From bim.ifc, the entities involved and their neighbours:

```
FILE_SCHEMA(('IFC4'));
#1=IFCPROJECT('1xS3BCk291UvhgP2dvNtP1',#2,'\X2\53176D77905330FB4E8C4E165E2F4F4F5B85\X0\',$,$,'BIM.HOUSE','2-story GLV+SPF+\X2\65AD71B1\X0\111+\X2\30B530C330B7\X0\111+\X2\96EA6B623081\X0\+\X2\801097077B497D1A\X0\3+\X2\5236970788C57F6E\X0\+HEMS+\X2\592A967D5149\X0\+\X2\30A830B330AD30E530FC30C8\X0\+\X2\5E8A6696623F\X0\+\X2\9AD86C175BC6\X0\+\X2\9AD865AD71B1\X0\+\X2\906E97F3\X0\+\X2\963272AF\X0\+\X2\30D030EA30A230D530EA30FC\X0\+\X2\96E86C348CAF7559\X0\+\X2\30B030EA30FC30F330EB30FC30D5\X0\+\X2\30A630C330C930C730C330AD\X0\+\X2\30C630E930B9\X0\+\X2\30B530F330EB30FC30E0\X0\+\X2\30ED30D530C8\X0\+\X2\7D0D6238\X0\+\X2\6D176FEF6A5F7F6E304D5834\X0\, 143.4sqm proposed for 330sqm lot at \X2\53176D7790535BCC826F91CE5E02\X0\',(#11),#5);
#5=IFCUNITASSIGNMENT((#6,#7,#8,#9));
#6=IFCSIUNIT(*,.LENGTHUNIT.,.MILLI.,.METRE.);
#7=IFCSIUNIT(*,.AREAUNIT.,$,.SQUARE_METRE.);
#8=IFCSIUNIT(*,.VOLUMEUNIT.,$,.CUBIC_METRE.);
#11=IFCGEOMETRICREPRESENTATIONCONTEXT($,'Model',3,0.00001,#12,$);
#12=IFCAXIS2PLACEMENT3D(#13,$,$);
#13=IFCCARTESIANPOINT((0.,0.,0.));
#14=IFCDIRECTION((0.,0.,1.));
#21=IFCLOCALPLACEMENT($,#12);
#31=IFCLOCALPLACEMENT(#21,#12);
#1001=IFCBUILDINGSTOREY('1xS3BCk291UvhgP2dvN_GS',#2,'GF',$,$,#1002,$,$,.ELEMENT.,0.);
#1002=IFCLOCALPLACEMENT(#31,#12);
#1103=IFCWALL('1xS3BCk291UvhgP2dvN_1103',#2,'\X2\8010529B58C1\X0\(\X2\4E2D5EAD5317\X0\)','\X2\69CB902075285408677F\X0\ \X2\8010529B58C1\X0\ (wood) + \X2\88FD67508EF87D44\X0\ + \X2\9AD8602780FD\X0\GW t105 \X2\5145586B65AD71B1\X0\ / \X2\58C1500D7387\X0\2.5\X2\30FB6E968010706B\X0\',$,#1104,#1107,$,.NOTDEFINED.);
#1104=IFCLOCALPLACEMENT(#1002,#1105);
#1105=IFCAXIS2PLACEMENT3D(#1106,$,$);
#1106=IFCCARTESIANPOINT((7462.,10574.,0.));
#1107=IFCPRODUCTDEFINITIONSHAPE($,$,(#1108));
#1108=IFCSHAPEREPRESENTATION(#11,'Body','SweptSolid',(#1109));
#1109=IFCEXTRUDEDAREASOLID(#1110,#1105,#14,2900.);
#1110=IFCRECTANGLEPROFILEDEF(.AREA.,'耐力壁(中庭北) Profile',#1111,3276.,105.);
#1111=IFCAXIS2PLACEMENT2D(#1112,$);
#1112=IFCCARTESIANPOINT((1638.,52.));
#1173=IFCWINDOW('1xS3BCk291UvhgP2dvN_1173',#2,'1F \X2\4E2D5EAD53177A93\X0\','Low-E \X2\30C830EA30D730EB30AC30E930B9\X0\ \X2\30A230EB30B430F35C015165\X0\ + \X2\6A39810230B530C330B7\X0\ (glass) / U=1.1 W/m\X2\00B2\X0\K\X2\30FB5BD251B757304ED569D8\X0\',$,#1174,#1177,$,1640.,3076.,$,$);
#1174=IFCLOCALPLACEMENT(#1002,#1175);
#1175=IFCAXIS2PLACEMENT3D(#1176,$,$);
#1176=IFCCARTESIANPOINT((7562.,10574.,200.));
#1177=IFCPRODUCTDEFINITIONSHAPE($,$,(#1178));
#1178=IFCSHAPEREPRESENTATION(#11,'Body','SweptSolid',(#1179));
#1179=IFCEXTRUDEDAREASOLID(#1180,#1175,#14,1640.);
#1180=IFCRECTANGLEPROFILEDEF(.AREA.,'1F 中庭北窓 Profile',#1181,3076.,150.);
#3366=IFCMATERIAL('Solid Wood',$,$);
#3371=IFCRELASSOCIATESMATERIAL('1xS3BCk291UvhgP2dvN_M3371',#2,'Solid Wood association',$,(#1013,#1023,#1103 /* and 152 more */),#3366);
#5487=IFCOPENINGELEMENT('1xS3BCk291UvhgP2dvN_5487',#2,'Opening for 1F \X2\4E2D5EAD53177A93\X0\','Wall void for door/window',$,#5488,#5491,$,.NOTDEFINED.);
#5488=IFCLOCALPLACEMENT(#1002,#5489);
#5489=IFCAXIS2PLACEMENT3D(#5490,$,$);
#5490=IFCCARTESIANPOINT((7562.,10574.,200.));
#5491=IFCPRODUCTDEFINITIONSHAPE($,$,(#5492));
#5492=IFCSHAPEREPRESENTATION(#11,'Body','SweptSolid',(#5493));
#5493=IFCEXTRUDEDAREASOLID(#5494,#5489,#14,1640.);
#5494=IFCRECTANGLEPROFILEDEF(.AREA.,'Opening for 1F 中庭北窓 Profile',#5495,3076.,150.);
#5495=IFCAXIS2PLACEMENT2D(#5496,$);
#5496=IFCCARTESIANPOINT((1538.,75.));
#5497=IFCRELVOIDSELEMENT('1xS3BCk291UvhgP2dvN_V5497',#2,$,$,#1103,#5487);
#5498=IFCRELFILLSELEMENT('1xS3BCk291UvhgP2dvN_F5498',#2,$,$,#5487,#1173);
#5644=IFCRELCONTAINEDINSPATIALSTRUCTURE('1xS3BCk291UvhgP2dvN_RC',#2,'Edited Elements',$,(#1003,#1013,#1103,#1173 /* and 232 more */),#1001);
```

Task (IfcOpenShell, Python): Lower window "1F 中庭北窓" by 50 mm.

```python
import numpy as np
import ifcopenshell
import ifcopenshell.api.geometry
import ifcopenshell.util.placement
import ifcopenshell.util.unit

model = ifcopenshell.open("bim.ifc")
unit_scale = ifcopenshell.util.unit.calculate_unit_scale(model)

window = model.by_guid("1xS3BCk291UvhgP2dvN_1173")
opening = window.FillsVoids[0].RelatingOpeningElement
dz = -0.05 / unit_scale

shift = np.array([0.0, 0.0, dz])
# The window is not placed relative to its opening, so move both.
for product in (opening, window):
    matrix = ifcopenshell.util.placement.get_local_placement(product.ObjectPlacement)
    matrix[:3, 3] += shift
    ifcopenshell.api.geometry.edit_object_placement(model, product=product, matrix=matrix, is_si=False)

print(f"moved by {dz * unit_scale:+.3f} m")

model.write("bim_edited.ifc")
```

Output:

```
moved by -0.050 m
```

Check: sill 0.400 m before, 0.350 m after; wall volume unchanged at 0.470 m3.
